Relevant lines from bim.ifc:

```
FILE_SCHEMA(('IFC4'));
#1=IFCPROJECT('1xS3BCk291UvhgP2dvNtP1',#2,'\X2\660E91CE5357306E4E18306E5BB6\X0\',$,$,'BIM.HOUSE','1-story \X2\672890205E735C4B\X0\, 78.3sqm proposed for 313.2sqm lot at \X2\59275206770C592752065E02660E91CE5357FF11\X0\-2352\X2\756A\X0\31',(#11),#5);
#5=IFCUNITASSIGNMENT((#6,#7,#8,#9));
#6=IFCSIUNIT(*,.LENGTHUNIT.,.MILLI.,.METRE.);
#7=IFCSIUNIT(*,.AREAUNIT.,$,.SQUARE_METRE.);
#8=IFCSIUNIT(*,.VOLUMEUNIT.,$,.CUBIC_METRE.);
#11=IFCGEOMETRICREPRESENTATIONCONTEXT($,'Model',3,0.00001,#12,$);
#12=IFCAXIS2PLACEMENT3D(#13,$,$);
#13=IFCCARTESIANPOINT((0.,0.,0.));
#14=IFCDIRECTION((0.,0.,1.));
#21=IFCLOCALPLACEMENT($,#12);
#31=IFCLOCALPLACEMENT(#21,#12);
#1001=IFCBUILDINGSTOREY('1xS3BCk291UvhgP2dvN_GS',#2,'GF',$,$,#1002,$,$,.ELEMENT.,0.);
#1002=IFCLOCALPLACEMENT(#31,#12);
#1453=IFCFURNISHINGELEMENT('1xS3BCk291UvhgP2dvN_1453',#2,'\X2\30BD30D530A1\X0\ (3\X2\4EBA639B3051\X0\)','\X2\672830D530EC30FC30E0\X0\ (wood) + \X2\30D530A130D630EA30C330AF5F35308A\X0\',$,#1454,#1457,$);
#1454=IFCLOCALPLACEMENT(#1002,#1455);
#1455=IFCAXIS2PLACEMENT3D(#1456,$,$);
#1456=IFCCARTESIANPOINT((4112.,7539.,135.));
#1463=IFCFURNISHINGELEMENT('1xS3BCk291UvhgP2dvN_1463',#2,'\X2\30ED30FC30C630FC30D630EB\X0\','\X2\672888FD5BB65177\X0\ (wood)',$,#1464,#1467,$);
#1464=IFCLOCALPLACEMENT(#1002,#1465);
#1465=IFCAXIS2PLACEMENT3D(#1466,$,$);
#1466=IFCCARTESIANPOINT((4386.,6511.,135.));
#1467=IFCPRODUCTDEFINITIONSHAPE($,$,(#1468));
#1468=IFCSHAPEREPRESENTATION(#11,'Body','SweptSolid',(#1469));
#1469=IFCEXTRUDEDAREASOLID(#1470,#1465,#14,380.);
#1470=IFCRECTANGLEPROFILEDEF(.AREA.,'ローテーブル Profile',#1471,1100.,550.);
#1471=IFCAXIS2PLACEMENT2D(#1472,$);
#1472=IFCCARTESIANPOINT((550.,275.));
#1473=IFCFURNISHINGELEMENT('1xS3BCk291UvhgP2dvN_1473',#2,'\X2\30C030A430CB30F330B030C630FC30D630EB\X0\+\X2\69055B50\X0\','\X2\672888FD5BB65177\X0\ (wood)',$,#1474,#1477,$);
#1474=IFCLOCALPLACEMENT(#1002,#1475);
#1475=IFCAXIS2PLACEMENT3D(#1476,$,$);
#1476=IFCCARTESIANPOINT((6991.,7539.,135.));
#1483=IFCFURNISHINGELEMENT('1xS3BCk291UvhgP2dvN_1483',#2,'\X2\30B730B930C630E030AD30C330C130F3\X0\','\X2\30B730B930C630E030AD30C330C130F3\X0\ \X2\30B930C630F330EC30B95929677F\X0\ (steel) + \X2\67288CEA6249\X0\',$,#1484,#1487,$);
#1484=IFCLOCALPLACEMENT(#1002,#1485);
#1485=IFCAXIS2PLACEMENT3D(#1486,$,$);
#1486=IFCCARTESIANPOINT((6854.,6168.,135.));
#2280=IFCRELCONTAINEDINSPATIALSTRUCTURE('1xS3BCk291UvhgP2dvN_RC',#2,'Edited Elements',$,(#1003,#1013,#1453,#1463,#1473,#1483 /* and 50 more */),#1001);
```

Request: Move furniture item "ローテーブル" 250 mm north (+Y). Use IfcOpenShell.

```python
import ifcopenshell
import ifcopenshell.api.geometry
import ifcopenshell.util.placement

model = ifcopenshell.open("bim.ifc")

item = model.by_guid("1xS3BCk291UvhgP2dvN_1463")
matrix = ifcopenshell.util.placement.get_local_placement(item.ObjectPlacement)
matrix[1, 3] += 250.0
ifcopenshell.api.geometry.edit_object_placement(model, product=item, matrix=matrix, is_si=False)

print(ifcopenshell.util.placement.get_local_placement(item.ObjectPlacement).round(3) + 0.0)

model.write("bim_updated.ifc")
```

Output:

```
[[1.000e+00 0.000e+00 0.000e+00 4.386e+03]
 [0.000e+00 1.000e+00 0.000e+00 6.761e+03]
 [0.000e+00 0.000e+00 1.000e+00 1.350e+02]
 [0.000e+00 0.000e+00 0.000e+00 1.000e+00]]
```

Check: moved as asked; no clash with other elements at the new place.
